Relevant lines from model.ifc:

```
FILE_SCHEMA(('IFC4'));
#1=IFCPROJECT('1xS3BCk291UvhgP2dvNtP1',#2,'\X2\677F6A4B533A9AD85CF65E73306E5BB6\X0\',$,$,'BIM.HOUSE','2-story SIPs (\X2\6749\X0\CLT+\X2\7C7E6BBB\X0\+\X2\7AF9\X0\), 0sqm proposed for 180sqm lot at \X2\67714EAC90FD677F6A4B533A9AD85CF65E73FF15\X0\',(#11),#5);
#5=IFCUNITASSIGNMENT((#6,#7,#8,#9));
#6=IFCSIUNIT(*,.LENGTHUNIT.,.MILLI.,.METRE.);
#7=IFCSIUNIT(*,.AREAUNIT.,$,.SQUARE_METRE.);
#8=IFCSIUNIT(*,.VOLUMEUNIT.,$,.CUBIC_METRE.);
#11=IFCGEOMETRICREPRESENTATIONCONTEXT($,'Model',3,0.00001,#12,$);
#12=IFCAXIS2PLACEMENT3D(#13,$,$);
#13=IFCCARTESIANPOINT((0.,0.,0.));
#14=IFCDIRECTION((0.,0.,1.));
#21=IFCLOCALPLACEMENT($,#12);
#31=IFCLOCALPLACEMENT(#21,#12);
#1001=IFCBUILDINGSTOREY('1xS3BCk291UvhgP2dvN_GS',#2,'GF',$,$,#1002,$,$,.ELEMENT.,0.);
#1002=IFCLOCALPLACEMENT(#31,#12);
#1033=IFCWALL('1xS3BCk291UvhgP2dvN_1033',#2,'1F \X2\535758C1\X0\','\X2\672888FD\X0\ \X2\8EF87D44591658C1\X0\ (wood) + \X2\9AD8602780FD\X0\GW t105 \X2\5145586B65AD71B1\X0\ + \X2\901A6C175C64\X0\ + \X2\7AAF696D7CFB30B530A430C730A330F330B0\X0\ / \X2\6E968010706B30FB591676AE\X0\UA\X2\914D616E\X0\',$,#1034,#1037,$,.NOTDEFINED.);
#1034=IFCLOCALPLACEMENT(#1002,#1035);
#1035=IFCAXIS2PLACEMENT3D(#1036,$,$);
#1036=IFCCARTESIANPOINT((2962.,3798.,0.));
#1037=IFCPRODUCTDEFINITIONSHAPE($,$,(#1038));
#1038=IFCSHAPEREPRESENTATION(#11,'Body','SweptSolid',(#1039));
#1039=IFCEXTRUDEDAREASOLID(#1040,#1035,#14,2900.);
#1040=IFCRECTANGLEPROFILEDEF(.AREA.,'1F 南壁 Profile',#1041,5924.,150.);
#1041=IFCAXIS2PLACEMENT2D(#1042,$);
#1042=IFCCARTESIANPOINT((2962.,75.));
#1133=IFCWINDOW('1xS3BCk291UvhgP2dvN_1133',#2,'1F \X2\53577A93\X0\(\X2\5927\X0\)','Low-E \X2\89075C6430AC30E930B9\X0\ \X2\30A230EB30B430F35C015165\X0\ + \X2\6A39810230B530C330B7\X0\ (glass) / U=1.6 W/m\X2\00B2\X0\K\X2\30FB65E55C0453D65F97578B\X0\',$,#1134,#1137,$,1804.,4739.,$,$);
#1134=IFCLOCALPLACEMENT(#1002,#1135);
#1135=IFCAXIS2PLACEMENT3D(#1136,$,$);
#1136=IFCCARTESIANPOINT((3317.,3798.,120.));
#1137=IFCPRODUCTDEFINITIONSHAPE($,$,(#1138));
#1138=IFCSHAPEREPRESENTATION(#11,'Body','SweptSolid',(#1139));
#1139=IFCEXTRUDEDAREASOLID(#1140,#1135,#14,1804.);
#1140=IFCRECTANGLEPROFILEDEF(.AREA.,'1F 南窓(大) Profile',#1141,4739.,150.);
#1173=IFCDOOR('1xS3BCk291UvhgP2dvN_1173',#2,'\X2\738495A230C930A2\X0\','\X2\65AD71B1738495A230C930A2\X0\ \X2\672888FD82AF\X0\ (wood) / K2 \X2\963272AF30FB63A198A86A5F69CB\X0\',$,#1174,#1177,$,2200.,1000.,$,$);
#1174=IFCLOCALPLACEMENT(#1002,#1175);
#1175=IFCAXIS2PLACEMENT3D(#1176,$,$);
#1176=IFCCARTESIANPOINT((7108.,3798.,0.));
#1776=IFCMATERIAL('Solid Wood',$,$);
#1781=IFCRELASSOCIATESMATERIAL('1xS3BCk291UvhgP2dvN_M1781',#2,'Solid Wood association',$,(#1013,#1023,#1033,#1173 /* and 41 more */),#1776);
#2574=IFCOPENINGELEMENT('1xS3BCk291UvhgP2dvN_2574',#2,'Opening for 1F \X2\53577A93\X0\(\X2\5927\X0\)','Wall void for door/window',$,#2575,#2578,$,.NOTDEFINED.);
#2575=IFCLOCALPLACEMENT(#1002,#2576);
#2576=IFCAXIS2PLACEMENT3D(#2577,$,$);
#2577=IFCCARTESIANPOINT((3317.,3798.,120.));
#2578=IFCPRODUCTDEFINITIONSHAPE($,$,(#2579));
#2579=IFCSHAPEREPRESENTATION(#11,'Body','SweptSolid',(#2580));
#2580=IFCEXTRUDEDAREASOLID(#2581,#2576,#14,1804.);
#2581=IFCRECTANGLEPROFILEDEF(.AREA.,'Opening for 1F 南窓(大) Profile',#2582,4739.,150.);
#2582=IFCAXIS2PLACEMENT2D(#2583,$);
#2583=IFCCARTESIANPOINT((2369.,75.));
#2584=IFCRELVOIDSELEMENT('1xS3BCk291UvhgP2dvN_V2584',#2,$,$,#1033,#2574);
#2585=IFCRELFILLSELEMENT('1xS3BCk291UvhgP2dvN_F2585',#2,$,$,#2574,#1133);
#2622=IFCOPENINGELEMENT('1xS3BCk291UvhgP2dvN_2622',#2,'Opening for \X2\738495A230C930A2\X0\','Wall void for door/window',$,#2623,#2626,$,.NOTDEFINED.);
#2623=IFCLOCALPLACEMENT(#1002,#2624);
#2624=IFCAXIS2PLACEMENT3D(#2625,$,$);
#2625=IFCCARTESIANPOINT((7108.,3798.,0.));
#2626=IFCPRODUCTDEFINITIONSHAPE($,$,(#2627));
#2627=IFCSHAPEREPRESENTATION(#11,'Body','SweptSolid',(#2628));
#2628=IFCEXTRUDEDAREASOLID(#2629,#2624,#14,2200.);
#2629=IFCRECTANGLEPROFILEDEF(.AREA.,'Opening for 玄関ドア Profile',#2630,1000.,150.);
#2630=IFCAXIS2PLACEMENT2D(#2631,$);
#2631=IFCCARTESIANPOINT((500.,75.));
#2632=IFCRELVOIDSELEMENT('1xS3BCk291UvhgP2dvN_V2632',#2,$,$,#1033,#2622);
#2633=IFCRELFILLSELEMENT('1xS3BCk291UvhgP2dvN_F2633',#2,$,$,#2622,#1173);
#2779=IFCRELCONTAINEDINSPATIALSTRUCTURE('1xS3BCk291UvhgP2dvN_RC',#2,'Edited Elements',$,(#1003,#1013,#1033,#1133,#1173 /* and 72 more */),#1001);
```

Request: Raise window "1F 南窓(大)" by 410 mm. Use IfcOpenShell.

```python
import numpy as np
import ifcopenshell
import ifcopenshell.api.geometry
import ifcopenshell.util.placement
import ifcopenshell.util.unit

model = ifcopenshell.open("model.ifc")
unit_scale = ifcopenshell.util.unit.calculate_unit_scale(model)

window = model.by_id(1133)
opening = window.FillsVoids[0].RelatingOpeningElement
dz = 410.0

shift = np.array([0.0, 0.0, dz])
# The window is not placed relative to its opening, so move both.
for product in (opening, window):
    matrix = ifcopenshell.util.placement.get_local_placement(product.ObjectPlacement)
    matrix[:3, 3] += shift
    ifcopenshell.api.geometry.edit_object_placement(model, product=product, matrix=matrix, is_si=False)

print(f"moved by {dz * unit_scale:+.3f} m")

model.write("model_rev.ifc")
```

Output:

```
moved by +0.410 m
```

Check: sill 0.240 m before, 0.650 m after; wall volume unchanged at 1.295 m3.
